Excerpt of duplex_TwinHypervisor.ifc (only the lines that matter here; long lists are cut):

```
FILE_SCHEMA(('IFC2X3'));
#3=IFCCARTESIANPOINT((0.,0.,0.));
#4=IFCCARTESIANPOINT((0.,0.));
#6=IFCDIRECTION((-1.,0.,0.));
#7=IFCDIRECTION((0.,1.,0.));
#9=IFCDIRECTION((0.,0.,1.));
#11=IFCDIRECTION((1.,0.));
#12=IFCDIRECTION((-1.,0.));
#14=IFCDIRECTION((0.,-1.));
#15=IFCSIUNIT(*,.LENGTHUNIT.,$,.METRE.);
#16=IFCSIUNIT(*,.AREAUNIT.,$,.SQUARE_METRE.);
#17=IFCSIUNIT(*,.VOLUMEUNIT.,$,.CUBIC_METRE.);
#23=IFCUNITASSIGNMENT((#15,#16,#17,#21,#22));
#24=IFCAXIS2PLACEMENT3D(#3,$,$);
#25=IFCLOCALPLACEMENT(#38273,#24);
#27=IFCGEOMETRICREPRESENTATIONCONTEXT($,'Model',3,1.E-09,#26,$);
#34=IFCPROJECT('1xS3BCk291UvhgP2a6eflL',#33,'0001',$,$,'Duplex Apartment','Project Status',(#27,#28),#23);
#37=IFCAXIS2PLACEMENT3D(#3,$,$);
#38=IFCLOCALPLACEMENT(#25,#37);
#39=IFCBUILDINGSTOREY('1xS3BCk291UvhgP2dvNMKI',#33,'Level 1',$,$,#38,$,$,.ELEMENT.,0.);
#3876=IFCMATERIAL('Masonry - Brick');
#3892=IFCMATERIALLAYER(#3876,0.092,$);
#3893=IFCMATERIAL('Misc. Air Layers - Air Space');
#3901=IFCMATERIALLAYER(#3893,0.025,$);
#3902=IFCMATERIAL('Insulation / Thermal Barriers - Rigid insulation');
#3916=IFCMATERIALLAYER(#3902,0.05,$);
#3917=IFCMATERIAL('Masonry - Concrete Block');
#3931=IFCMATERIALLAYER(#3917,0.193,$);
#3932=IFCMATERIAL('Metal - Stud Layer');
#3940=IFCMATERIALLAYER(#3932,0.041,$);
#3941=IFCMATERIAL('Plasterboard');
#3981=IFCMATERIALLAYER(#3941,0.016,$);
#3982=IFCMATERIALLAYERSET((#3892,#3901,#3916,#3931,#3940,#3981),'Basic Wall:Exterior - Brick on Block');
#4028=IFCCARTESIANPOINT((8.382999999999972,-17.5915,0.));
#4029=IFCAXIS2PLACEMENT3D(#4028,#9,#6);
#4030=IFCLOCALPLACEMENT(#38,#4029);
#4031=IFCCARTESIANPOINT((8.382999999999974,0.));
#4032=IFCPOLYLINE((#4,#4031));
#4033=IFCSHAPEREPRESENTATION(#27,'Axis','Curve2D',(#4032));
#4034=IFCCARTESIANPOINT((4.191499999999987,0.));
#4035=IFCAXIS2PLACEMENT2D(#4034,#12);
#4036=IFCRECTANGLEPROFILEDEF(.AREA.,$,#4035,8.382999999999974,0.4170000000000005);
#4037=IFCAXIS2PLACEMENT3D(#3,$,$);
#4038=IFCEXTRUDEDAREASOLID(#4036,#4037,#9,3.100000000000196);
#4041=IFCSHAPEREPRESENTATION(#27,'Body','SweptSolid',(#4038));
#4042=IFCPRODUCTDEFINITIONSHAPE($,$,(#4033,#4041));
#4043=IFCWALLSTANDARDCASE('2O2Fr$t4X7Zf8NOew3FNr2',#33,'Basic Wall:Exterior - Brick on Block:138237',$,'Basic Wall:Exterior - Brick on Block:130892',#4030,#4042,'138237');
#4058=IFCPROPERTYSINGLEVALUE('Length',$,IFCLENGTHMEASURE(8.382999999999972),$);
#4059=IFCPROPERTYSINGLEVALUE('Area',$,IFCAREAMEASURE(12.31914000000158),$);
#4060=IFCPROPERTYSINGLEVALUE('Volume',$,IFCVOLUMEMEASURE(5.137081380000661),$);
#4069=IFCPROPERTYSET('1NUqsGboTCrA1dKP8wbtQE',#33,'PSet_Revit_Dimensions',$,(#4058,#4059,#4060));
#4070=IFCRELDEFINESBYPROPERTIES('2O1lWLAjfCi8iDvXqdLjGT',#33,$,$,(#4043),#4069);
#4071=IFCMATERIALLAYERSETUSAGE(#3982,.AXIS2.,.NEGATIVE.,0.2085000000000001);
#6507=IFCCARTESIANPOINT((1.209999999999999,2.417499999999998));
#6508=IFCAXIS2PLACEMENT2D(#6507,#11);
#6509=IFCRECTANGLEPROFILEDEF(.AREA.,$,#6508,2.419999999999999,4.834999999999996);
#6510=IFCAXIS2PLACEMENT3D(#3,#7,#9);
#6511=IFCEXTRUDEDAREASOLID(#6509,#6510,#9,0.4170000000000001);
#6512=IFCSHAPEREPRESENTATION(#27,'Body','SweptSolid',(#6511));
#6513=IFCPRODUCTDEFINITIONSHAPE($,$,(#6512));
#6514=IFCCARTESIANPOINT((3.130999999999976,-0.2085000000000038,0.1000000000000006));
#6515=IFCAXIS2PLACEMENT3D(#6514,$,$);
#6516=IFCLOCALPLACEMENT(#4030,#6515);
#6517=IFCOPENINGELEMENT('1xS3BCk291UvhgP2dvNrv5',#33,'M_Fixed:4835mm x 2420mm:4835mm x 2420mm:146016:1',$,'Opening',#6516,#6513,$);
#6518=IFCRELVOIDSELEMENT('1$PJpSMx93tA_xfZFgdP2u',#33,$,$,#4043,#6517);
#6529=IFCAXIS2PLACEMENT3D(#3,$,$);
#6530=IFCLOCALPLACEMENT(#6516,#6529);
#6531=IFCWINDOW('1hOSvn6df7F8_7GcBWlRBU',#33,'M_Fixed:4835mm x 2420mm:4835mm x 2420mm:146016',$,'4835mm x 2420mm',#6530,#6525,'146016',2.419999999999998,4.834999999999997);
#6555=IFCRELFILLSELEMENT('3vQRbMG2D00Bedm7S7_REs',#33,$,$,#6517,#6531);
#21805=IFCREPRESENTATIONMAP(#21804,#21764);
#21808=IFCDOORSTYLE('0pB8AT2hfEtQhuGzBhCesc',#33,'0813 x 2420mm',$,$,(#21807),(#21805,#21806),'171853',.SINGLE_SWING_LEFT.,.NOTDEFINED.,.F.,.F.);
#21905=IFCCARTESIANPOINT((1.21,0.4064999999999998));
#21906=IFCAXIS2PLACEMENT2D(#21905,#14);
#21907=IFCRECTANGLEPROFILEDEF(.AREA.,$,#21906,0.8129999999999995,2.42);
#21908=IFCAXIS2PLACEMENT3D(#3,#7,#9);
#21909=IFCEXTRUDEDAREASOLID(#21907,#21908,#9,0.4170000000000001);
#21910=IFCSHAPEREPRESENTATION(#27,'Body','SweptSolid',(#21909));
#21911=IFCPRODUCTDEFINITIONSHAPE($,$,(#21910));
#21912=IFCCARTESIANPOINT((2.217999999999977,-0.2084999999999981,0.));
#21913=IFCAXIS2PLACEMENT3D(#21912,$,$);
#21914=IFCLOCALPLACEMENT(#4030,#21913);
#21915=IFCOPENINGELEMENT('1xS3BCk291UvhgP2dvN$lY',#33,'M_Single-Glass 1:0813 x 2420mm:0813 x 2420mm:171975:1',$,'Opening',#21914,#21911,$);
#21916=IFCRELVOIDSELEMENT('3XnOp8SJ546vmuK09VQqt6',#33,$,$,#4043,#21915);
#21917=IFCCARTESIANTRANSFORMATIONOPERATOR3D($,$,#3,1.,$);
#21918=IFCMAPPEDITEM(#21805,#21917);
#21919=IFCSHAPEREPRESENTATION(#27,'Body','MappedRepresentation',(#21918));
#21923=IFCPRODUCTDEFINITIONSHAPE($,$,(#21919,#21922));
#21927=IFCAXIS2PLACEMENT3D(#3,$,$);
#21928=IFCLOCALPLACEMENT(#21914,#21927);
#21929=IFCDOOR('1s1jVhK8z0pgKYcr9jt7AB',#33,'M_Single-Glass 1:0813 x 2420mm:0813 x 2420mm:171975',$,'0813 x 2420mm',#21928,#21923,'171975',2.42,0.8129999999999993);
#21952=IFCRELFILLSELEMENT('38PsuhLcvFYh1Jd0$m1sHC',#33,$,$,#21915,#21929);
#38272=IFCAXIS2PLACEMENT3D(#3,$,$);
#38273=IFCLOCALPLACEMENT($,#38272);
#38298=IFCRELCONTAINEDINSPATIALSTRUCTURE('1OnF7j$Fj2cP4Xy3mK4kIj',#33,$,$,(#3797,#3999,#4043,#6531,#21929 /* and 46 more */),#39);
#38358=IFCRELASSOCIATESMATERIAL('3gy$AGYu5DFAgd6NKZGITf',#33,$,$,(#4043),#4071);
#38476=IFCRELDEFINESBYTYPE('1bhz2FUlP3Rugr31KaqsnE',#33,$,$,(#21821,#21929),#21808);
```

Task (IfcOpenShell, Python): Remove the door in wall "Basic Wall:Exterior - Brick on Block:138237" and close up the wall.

```python
import ifcopenshell
import ifcopenshell.api.feature
import ifcopenshell.api.pset
import ifcopenshell.api.root
import ifcopenshell.geom
import ifcopenshell.util.element
import ifcopenshell.util.shape
import ifcopenshell.util.unit

model = ifcopenshell.open("duplex_TwinHypervisor.ifc")
area_scale = ifcopenshell.util.unit.calculate_unit_scale(model, "AREAUNIT")
volume_scale = ifcopenshell.util.unit.calculate_unit_scale(model, "VOLUMEUNIT")
settings = ifcopenshell.geom.settings()


def volume(element):
    """Net volume in cubic metres, openings subtracted."""
    shape = ifcopenshell.geom.create_shape(settings, element)
    return ifcopenshell.util.shape.get_volume(shape.geometry)


door = model.by_guid("1s1jVhK8z0pgKYcr9jt7AB")
opening = door.FillsVoids[0].RelatingOpeningElement
wall = opening.VoidsElements[0].RelatingBuildingElement
before = volume(wall)

ifcopenshell.api.root.remove_product(model, product=door)
ifcopenshell.api.feature.remove_feature(model, feature=opening)

after = volume(wall)
thickness = 0.417  # wall thickness in metres

# Update the wall's stored quantities.
pset = model.by_id(ifcopenshell.util.element.get_pset(wall, "PSet_Revit_Dimensions", should_inherit=False)["id"])
ifcopenshell.api.pset.edit_pset(model, pset=pset, properties={
    "Area": model.create_entity("IfcAreaMeasure", after / thickness / area_scale),
    "Volume": model.create_entity("IfcVolumeMeasure", after / volume_scale),
})

print(f"wall volume {before:.3f} -> {after:.3f} m3")

model.write("duplex_TwinHypervisor_v2.ifc")
```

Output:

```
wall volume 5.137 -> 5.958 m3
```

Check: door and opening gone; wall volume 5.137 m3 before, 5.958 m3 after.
